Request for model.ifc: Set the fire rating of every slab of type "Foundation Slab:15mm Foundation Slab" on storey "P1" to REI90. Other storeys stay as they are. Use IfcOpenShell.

First a look at what the model holds.

```python
import ifcopenshell
import ifcopenshell.util.element

model = ifcopenshell.open("model.ifc")
print(model.schema)
storey = next(s for s in model.by_type("IfcBuildingStorey") if s.Name == "P1")
slabs = [e for e in ifcopenshell.util.element.get_decomposition(storey) if e.is_a("IfcSlab")]
seen = {}
for e in slabs:
    element_type = ifcopenshell.util.element.get_type(e)
    key = (element_type.Name if element_type != e and element_type else None, ifcopenshell.util.element.get_pset(e, "Pset_SlabCommon", "FireRating"))
    seen[key] = seen.get(key, 0) + 1
for (name, value), count in sorted(seen.items(), key=str):
    print(count, "x", name, "|", value)
```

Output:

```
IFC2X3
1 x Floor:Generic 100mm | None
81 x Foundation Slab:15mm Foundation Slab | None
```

```python
import ifcopenshell
import ifcopenshell.api.pset
import ifcopenshell.util.element

model = ifcopenshell.open("model.ifc")

storey = next(s for s in model.by_type("IfcBuildingStorey") if s.Name == "P1")
slabs = [e for e in ifcopenshell.util.element.get_decomposition(storey) if e.is_a("IfcSlab")]

count = 0
for e in slabs:
    element_type = ifcopenshell.util.element.get_type(e)
    if element_type in (None, e) or element_type.Name != "Foundation Slab:15mm Foundation Slab":
        continue
    # add_pset returns the element's existing set when there is one.
    pset = ifcopenshell.api.pset.add_pset(model, product=e, name="Pset_SlabCommon")
    ifcopenshell.api.pset.edit_pset(model, pset=pset, properties={"FireRating": "REI90"})
    count += 1

print(count, "slabs updated")

model.write("model_updated.ifc")
```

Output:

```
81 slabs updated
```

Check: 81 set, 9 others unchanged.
